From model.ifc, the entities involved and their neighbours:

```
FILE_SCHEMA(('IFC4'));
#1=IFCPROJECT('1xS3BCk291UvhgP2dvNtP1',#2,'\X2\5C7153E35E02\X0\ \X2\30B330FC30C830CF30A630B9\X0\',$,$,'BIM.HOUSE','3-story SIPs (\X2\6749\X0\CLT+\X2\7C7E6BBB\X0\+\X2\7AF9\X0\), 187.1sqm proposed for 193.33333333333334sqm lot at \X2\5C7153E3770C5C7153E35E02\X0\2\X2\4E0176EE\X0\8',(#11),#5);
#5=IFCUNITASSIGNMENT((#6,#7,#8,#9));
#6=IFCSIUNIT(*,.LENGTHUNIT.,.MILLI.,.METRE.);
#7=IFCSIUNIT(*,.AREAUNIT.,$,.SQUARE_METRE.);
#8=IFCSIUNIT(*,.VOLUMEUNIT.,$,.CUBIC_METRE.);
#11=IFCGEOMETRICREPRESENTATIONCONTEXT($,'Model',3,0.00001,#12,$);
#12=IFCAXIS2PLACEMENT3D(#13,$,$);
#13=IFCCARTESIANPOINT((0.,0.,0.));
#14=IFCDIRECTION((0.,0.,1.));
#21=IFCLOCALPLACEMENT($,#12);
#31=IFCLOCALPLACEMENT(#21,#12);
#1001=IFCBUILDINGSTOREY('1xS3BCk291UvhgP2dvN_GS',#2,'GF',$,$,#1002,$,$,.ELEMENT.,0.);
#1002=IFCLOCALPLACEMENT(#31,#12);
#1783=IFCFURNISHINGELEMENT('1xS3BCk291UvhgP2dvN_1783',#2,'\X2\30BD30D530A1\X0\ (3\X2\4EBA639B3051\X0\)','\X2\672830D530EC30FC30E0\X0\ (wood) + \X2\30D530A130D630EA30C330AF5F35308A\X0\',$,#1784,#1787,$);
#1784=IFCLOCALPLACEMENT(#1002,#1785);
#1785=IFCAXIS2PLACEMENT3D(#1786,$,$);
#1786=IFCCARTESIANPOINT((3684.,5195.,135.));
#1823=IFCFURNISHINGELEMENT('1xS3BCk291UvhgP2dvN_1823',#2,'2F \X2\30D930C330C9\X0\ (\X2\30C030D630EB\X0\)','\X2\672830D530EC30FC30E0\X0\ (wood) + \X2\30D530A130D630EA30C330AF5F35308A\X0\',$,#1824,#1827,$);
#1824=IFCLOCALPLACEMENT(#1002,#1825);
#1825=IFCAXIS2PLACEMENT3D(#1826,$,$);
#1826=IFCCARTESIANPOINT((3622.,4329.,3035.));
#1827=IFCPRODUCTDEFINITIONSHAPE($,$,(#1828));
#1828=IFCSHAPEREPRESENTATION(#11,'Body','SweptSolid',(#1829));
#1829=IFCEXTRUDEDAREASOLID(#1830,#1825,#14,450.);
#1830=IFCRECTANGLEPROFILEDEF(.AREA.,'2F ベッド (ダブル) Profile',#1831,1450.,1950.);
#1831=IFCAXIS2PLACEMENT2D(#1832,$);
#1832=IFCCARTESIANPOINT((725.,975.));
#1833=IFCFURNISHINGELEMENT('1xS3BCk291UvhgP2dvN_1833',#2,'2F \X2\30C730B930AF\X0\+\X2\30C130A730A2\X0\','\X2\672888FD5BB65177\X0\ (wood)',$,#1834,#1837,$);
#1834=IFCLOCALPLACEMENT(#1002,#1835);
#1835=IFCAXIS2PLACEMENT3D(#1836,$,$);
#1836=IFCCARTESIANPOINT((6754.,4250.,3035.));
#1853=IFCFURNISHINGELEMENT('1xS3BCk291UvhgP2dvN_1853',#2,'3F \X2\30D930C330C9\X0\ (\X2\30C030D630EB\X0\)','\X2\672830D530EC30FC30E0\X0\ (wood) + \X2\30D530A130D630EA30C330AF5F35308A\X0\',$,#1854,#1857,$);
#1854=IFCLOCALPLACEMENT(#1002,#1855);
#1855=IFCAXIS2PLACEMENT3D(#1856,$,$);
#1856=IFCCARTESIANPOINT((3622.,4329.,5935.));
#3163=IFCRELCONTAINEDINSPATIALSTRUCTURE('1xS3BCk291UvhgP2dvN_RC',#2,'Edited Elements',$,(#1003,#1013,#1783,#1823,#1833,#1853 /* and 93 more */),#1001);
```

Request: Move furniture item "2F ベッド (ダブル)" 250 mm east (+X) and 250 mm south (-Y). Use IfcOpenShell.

```python
import ifcopenshell
import ifcopenshell.api.geometry
import ifcopenshell.util.placement

model = ifcopenshell.open("model.ifc")

item = model.by_id(1823)
matrix = ifcopenshell.util.placement.get_local_placement(item.ObjectPlacement)
matrix[0, 3] += 250.0
matrix[1, 3] -= 250.0
ifcopenshell.api.geometry.edit_object_placement(model, product=item, matrix=matrix, is_si=False)

print(ifcopenshell.util.placement.get_local_placement(item.ObjectPlacement).round(3) + 0.0)

model.write("model-out.ifc")
```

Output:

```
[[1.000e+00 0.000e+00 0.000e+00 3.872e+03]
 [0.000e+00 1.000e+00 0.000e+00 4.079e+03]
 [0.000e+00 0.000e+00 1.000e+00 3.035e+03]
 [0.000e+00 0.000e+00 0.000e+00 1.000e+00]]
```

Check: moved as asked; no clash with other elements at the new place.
